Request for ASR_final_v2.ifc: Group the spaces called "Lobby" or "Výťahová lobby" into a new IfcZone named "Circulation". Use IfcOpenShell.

First a look at what the model holds.

```python
import ifcopenshell

model = ifcopenshell.open("ASR_final_v2.ifc")
print(model.schema)
seen = {}
for space in model.by_type("IfcSpace"):
    seen[space.LongName] = seen.get(space.LongName, 0) + 1
for name, count in sorted(seen.items(), key=str):
    print(count, "x", name)
print("zones:", [z.Name for z in model.by_type("IfcZone")][:20])
```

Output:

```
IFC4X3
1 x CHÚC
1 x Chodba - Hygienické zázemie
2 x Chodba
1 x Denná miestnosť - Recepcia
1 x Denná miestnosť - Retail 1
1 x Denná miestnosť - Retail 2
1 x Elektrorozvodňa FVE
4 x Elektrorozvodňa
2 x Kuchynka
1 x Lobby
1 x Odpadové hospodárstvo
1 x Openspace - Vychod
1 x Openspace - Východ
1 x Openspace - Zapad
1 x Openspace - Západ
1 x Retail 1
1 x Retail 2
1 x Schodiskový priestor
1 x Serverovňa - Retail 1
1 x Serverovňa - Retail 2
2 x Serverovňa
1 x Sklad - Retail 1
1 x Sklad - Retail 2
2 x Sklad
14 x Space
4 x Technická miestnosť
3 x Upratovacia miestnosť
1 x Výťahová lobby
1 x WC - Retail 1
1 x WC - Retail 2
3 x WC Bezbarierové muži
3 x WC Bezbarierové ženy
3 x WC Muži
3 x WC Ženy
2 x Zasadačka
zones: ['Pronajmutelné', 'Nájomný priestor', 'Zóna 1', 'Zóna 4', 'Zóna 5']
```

```python
import ifcopenshell
import ifcopenshell.api.group
import ifcopenshell.api.root

model = ifcopenshell.open("ASR_final_v2.ifc")

names = {"Lobby", "Výťahová lobby"}
spaces = [s for s in model.by_type("IfcSpace") if s.LongName in names]

zone = ifcopenshell.api.root.create_entity(model, ifc_class="IfcZone", name="Circulation")
ifcopenshell.api.group.assign_group(model, products=spaces, group=zone)
print(len(spaces), "spaces in", zone.Name)

model.write("ASR_final_v2-out.ifc")
```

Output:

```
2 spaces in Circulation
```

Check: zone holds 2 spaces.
